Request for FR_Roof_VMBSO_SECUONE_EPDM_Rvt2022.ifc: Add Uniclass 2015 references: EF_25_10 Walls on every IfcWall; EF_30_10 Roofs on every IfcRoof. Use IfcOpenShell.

First a look at what the model holds.

```python
import ifcopenshell

model = ifcopenshell.open("FR_Roof_VMBSO_SECUONE_EPDM_Rvt2022.ifc")
print(model.schema)
print("classifications:", [c.Name for c in model.by_type("IfcClassification")])
for ifc_class in ("IfcDoor", "IfcRoof", "IfcStair", "IfcWall", "IfcWindow"):
    print(ifc_class, len(model.by_type(ifc_class)))
```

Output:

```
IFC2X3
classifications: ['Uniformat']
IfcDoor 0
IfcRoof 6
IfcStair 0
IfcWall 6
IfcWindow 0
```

```python
import ifcopenshell
import ifcopenshell.api.classification

model = ifcopenshell.open("FR_Roof_VMBSO_SECUONE_EPDM_Rvt2022.ifc")

# IFC2X3 requires Source and Edition and has no link from the project to the system.
system = model.create_entity("IfcClassification", Source="NBS", Edition="2015", Name="Uniclass 2015")

codes = {
    "IfcWall": ("EF_25_10", "Walls"),
    "IfcRoof": ("EF_30_10", "Roofs"),
}
for ifc_class, (code, name) in codes.items():
    products = model.by_type(ifc_class)
    ifcopenshell.api.classification.add_reference(
        model, products=products, classification=system, identification=code, name=name
    )
    print(code, len(products))

model.write("FR_Roof_VMBSO_SECUONE_EPDM_Rvt2022_v2.ifc")
```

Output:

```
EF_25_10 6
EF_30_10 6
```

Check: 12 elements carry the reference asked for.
